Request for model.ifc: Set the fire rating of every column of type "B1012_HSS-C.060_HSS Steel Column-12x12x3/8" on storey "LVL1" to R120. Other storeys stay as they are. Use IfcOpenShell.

First a look at what the model holds.

```python
import ifcopenshell
import ifcopenshell.util.element

model = ifcopenshell.open("model.ifc")
print(model.schema)
storey = next(s for s in model.by_type("IfcBuildingStorey") if s.Name == "LVL1")
columns = [e for e in ifcopenshell.util.element.get_decomposition(storey) if e.is_a("IfcColumn")]
seen = {}
for e in columns:
    element_type = ifcopenshell.util.element.get_type(e)
    key = (element_type.Name if element_type != e and element_type else None, ifcopenshell.util.element.get_pset(e, "Pset_ColumnCommon", "FireRating"))
    seen[key] = seen.get(key, 0) + 1
for (name, value), count in sorted(seen.items(), key=str):
    print(count, "x", name, "|", value)
```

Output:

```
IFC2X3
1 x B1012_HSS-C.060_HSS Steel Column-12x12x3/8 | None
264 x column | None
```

```python
import ifcopenshell
import ifcopenshell.api.pset
import ifcopenshell.util.element

model = ifcopenshell.open("model.ifc")

storey = next(s for s in model.by_type("IfcBuildingStorey") if s.Name == "LVL1")
columns = [e for e in ifcopenshell.util.element.get_decomposition(storey) if e.is_a("IfcColumn")]

count = 0
for e in columns:
    element_type = ifcopenshell.util.element.get_type(e)
    if element_type in (None, e) or element_type.Name != "B1012_HSS-C.060_HSS Steel Column-12x12x3/8":
        continue
    # add_pset returns the element's existing set when there is one.
    pset = ifcopenshell.api.pset.add_pset(model, product=e, name="Pset_ColumnCommon")
    ifcopenshell.api.pset.edit_pset(model, pset=pset, properties={"FireRating": "R120"})
    count += 1

print(count, "columns updated")

model.write("model_updated.ifc")
```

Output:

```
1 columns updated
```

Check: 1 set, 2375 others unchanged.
